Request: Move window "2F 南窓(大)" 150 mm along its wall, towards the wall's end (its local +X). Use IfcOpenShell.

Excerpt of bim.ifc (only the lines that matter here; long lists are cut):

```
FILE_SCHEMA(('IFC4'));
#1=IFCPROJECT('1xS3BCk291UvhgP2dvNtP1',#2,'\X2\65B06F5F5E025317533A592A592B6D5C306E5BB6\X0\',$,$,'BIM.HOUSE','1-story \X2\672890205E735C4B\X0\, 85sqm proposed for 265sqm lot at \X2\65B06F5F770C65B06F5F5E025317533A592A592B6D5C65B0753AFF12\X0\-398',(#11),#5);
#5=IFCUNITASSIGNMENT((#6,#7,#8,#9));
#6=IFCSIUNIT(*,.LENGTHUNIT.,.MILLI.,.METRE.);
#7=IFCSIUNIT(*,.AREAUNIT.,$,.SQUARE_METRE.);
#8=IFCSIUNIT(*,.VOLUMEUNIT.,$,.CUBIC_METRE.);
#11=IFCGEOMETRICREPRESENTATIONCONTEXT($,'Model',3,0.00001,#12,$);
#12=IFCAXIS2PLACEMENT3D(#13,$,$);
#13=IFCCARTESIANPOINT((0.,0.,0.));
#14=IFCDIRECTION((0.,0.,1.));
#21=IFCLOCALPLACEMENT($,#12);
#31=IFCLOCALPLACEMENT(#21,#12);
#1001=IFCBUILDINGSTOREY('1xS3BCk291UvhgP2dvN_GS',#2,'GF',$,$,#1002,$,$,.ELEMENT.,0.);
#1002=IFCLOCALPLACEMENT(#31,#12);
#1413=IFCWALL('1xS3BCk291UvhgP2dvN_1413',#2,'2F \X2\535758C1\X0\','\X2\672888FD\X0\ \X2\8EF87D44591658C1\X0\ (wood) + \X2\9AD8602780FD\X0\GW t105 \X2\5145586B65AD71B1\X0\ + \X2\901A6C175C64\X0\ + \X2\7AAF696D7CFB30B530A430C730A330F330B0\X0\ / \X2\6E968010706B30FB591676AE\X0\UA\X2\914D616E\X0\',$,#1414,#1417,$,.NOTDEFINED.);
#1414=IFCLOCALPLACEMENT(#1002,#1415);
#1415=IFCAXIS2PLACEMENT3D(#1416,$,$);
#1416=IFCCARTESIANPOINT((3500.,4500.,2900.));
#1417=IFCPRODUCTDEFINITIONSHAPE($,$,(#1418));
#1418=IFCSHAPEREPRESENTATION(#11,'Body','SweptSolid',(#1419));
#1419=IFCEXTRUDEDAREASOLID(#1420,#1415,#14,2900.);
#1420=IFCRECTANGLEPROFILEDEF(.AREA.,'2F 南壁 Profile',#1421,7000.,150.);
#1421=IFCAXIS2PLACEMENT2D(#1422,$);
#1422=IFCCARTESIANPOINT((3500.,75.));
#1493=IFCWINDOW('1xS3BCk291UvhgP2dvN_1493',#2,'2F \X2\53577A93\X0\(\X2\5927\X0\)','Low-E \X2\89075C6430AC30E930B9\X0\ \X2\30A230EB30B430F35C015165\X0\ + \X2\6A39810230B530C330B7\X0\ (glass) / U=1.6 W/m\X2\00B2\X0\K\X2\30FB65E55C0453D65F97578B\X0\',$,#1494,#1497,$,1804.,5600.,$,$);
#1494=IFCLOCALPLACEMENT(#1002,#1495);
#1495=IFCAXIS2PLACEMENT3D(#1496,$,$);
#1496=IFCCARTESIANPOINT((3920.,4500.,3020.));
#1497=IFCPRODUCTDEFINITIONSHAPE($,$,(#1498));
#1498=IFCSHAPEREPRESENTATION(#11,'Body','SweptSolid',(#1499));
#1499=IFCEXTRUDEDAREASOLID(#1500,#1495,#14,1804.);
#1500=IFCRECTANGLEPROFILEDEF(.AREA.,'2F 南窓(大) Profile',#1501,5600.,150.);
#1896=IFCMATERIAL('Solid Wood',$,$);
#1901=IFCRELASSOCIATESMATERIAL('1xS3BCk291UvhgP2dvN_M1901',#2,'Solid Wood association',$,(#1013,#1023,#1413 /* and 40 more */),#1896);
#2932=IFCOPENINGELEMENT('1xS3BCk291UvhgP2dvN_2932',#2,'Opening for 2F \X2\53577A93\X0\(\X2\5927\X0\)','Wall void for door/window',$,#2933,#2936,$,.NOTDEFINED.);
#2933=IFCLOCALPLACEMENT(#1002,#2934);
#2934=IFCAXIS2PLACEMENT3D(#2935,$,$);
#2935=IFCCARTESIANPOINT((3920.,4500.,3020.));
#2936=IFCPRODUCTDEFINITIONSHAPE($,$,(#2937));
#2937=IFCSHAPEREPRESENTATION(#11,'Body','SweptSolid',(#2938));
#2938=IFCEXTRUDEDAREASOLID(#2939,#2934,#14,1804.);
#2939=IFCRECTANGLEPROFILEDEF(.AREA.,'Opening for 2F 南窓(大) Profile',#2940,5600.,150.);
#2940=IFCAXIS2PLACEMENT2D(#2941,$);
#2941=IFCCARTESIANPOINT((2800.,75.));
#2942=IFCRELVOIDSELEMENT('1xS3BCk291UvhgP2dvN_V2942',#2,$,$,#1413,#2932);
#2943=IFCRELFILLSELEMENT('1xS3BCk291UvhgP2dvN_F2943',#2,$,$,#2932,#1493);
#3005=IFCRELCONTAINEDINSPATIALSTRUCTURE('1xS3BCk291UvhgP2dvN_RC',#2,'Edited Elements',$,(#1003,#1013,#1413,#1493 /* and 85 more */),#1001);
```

```python
import ifcopenshell
import ifcopenshell.api.geometry
import ifcopenshell.util.placement

model = ifcopenshell.open("bim.ifc")

window = model.by_id(1493)
opening = window.FillsVoids[0].RelatingOpeningElement
wall = opening.VoidsElements[0].RelatingBuildingElement

wall_matrix = ifcopenshell.util.placement.get_local_placement(wall.ObjectPlacement)
shift = wall_matrix[:3, 0] * 150.0
before = ifcopenshell.util.placement.get_local_placement(window.ObjectPlacement)[:3, 3].copy()

# The window is not placed relative to its opening, so move both.
for product in (opening, window):
    matrix = ifcopenshell.util.placement.get_local_placement(product.ObjectPlacement)
    matrix[:3, 3] += shift
    ifcopenshell.api.geometry.edit_object_placement(model, product=product, matrix=matrix, is_si=False)

after = ifcopenshell.util.placement.get_local_placement(window.ObjectPlacement)[:3, 3]
print("window moved by", (after - before).round(3) + 0.0)

model.write("bim_edited.ifc")
```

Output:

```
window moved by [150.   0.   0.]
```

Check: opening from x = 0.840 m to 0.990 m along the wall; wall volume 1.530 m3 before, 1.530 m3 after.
